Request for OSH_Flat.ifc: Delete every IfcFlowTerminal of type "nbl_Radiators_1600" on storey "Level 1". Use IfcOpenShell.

First a look at what the model holds.

```python
import ifcopenshell
import ifcopenshell.util.element

model = ifcopenshell.open("OSH_Flat.ifc")
print(model.schema)
storey = next(s for s in model.by_type("IfcBuildingStorey") if s.Name == "Level 1")
terminals = [e for e in ifcopenshell.util.element.get_decomposition(storey) if e.is_a("IfcFlowTerminal")]
seen = {}
for e in terminals:
    element_type = ifcopenshell.util.element.get_type(e)
    name = element_type.Name if element_type not in (None, e) else None
    seen[name] = seen.get(name, 0) + 1
for name, count in sorted(seen.items(), key=str):
    print(count, "x", name)
```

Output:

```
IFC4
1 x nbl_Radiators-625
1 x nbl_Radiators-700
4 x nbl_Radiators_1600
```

```python
import ifcopenshell
import ifcopenshell.api.root
import ifcopenshell.util.element

model = ifcopenshell.open("OSH_Flat.ifc")

storey = next(s for s in model.by_type("IfcBuildingStorey") if s.Name == "Level 1")
terminals = [e for e in ifcopenshell.util.element.get_decomposition(storey) if e.is_a("IfcFlowTerminal")]
targets = [e for e in terminals if (t := ifcopenshell.util.element.get_type(e)) not in (None, e) and t.Name == "nbl_Radiators_1600"]

for e in targets:
    ifcopenshell.api.root.remove_product(model, product=e)
print(len(targets), "removed")

model.write("OSH_Flat_v2.ifc")
```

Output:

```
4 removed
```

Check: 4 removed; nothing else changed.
